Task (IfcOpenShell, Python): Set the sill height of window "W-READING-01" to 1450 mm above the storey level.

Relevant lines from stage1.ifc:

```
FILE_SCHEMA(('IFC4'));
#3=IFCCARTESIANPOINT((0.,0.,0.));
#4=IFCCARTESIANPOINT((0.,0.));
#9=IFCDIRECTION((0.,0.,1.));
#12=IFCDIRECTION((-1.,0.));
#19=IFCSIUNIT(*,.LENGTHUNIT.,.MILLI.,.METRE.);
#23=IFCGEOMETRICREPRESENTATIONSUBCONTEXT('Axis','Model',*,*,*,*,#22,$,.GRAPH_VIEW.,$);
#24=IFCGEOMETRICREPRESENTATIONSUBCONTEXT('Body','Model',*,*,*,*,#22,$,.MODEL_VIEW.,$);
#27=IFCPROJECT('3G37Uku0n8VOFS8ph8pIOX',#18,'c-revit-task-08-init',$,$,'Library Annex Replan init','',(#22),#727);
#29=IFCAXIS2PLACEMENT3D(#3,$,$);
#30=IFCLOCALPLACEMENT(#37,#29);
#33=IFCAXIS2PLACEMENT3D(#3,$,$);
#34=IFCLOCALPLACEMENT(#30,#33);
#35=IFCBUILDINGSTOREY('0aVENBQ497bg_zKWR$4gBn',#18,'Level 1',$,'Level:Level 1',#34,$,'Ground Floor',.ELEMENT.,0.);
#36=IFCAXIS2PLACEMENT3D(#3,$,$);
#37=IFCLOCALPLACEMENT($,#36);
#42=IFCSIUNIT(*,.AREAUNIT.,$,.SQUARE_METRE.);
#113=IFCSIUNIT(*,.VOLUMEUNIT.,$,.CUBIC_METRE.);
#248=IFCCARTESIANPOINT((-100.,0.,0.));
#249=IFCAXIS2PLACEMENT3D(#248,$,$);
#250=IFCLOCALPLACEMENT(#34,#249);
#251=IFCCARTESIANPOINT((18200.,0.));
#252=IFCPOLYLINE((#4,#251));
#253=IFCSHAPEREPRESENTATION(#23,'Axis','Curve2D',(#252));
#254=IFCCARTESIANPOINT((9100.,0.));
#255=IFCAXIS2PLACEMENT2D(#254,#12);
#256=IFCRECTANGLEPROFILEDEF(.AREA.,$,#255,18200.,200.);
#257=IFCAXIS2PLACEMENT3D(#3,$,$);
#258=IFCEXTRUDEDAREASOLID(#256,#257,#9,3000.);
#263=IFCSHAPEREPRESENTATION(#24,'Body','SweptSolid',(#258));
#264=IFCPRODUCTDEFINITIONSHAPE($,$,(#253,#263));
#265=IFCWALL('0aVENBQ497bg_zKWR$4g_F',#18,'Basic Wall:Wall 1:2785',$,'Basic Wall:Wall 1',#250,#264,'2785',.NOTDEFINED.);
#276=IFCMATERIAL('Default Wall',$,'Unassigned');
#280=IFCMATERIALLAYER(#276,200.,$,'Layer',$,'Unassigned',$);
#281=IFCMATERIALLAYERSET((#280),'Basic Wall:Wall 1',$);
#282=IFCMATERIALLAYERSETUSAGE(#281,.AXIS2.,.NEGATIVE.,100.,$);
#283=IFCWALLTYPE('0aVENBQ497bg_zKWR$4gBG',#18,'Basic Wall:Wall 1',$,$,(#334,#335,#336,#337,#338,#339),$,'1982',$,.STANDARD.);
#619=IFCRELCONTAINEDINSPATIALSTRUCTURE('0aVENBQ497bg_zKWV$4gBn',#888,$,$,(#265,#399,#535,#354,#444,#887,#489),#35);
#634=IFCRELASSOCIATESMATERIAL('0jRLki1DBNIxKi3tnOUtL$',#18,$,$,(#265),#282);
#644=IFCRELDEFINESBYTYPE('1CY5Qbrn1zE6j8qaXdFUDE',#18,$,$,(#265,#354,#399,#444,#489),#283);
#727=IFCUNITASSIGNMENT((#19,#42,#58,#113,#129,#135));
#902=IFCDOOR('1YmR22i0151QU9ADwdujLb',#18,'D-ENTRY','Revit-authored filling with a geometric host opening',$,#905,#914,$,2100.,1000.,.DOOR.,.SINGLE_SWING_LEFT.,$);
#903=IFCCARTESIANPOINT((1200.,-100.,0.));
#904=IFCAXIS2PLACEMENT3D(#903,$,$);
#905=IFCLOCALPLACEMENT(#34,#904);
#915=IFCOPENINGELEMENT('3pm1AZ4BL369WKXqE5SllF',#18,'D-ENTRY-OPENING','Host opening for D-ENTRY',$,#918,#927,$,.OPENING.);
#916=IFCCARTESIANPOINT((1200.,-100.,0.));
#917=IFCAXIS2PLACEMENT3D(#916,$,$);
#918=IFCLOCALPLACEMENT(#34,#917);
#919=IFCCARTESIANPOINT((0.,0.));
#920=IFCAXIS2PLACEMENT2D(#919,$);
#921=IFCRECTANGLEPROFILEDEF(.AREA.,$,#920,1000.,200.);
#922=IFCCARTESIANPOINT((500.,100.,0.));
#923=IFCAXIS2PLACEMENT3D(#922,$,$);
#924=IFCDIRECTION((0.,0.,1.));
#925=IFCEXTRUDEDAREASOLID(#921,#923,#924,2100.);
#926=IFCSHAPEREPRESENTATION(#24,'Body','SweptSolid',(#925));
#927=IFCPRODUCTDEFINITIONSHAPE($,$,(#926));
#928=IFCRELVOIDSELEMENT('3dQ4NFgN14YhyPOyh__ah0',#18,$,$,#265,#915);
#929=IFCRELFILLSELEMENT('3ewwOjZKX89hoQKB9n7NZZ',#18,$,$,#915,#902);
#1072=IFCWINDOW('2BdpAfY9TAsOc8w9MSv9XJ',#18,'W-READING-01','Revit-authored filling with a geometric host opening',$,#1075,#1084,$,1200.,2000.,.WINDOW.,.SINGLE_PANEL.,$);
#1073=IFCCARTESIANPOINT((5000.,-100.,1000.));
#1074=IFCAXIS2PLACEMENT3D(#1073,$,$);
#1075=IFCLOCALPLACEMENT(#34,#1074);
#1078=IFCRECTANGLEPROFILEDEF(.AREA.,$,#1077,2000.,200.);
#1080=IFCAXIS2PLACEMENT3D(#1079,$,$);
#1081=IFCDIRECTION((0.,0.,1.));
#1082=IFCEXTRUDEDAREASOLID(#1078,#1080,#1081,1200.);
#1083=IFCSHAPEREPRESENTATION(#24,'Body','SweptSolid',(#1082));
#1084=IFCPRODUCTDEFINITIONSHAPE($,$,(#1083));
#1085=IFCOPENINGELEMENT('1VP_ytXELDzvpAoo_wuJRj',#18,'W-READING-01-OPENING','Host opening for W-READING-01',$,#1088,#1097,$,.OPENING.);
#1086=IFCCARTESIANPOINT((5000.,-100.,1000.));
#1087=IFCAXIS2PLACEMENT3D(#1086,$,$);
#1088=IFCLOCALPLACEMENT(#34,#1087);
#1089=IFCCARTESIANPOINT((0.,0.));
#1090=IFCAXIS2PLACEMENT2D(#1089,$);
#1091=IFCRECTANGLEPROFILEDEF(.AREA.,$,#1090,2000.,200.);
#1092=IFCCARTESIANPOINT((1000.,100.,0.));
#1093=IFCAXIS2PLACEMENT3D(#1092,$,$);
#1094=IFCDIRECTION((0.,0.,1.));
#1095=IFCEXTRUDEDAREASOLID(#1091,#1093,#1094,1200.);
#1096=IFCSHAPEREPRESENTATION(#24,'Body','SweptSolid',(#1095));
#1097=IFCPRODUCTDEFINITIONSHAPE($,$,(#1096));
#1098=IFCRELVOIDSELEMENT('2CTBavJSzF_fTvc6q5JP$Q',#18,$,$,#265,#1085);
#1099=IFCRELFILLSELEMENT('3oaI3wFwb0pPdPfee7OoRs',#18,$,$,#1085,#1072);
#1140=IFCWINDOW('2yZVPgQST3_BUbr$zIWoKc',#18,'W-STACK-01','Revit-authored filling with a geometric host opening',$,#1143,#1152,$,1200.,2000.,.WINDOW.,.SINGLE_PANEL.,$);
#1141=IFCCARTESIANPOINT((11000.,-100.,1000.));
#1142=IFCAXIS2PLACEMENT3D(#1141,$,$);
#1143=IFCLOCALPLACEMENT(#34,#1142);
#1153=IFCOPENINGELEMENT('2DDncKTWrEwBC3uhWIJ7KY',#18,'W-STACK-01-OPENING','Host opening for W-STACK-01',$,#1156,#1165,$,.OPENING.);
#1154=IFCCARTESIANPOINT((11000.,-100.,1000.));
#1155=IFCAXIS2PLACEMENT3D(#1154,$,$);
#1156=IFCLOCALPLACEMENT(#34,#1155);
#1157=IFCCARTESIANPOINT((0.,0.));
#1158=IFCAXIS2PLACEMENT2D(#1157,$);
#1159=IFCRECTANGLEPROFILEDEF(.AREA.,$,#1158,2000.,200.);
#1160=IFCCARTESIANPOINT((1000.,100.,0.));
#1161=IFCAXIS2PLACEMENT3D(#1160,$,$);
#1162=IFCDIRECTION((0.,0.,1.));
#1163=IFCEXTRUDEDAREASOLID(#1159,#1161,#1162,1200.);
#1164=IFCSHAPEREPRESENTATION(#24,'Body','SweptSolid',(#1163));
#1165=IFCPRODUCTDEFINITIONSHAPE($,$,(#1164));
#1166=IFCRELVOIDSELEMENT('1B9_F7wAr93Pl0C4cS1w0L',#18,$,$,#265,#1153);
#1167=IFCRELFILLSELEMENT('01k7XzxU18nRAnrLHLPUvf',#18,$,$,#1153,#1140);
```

```python
import numpy as np
import ifcopenshell
import ifcopenshell.api.geometry
import ifcopenshell.geom
import ifcopenshell.util.element
import ifcopenshell.util.placement
import ifcopenshell.util.shape
import ifcopenshell.util.unit

model = ifcopenshell.open("stage1.ifc")
unit_scale = ifcopenshell.util.unit.calculate_unit_scale(model)

window = model.by_id(1072)
opening = window.FillsVoids[0].RelatingOpeningElement
storey = ifcopenshell.util.element.get_container(window, ifc_class="IfcBuildingStorey")
level = ifcopenshell.util.placement.get_local_placement(storey.ObjectPlacement)[2, 3]

# The opening's origin need not be at the sill, so measure its lowest point.
shape = ifcopenshell.geom.create_shape(ifcopenshell.geom.settings(), opening)
bottom = ifcopenshell.util.shape.get_shape_bottom_elevation(shape, shape.geometry) / unit_scale
dz = level + 1450.0 - bottom

shift = np.array([0.0, 0.0, dz])
# The window is not placed relative to its opening, so move both.
for product in (opening, window):
    matrix = ifcopenshell.util.placement.get_local_placement(product.ObjectPlacement)
    matrix[:3, 3] += shift
    ifcopenshell.api.geometry.edit_object_placement(model, product=product, matrix=matrix, is_si=False)

print(f"moved by {dz * unit_scale:+.3f} m")

model.write("stage1_updated.ifc")
```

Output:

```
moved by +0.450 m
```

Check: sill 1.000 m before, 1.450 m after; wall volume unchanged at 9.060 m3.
